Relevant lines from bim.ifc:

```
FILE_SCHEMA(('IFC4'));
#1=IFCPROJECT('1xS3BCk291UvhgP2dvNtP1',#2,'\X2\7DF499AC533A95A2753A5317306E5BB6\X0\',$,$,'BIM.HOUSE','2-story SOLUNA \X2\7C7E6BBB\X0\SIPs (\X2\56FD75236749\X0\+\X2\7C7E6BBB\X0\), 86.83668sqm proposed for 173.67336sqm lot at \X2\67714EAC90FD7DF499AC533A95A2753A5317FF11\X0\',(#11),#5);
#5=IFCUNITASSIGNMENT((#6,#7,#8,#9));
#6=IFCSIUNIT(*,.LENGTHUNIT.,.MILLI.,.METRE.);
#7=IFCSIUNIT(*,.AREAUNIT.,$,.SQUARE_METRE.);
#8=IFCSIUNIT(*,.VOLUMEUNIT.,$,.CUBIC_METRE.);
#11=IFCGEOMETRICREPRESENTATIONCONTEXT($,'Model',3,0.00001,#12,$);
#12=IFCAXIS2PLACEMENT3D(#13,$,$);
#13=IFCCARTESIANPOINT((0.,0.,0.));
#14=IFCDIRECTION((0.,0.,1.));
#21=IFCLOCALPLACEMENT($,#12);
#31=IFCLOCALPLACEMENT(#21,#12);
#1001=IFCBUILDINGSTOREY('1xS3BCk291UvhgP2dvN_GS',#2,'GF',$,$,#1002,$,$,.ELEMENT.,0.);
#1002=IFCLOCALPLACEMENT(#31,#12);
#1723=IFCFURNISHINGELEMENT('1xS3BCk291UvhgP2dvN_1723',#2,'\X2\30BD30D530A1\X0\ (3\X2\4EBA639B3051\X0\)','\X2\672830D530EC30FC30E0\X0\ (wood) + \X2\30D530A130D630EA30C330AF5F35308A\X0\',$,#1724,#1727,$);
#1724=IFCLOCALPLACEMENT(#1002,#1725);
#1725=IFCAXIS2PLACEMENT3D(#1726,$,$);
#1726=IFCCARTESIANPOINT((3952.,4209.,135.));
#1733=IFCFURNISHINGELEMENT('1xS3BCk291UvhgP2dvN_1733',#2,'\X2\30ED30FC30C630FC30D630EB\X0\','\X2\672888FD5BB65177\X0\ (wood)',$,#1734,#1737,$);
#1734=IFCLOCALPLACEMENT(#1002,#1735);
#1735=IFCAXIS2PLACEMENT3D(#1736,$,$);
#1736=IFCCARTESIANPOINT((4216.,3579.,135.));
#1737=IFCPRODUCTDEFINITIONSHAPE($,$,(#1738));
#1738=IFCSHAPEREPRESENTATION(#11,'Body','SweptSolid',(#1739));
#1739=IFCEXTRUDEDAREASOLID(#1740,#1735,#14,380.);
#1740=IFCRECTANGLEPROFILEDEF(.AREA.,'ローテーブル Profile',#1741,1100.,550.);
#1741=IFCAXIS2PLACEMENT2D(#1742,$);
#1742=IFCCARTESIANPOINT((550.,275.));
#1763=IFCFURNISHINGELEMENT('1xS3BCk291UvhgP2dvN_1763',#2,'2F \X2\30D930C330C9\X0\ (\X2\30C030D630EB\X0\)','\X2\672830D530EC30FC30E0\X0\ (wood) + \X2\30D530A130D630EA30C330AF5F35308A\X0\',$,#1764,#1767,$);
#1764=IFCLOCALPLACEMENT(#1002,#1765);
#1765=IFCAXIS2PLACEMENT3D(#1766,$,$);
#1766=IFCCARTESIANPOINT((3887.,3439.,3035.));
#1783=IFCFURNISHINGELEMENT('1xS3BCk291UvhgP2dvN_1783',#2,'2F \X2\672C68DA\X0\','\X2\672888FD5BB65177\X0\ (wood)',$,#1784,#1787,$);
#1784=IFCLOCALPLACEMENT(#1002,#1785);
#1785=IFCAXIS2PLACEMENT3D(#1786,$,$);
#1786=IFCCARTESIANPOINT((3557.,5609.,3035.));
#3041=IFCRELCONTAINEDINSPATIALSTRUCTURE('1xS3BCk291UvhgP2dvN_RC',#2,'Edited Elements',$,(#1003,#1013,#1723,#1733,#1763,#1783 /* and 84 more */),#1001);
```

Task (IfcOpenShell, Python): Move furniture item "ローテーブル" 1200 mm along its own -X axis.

```python
import ifcopenshell
import ifcopenshell.api.geometry
import ifcopenshell.util.placement

model = ifcopenshell.open("bim.ifc")

item = model.by_id(1733)
matrix = ifcopenshell.util.placement.get_local_placement(item.ObjectPlacement)
matrix[:3, 3] -= matrix[:3, 0] * 1200.0
ifcopenshell.api.geometry.edit_object_placement(model, product=item, matrix=matrix, is_si=False)

print(ifcopenshell.util.placement.get_local_placement(item.ObjectPlacement).round(3) + 0.0)

model.write("bim_updated.ifc")
```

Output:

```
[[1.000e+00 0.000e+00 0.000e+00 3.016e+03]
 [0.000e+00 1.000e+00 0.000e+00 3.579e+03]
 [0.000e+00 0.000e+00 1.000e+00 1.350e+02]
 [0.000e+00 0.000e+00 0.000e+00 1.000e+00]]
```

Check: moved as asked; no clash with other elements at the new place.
